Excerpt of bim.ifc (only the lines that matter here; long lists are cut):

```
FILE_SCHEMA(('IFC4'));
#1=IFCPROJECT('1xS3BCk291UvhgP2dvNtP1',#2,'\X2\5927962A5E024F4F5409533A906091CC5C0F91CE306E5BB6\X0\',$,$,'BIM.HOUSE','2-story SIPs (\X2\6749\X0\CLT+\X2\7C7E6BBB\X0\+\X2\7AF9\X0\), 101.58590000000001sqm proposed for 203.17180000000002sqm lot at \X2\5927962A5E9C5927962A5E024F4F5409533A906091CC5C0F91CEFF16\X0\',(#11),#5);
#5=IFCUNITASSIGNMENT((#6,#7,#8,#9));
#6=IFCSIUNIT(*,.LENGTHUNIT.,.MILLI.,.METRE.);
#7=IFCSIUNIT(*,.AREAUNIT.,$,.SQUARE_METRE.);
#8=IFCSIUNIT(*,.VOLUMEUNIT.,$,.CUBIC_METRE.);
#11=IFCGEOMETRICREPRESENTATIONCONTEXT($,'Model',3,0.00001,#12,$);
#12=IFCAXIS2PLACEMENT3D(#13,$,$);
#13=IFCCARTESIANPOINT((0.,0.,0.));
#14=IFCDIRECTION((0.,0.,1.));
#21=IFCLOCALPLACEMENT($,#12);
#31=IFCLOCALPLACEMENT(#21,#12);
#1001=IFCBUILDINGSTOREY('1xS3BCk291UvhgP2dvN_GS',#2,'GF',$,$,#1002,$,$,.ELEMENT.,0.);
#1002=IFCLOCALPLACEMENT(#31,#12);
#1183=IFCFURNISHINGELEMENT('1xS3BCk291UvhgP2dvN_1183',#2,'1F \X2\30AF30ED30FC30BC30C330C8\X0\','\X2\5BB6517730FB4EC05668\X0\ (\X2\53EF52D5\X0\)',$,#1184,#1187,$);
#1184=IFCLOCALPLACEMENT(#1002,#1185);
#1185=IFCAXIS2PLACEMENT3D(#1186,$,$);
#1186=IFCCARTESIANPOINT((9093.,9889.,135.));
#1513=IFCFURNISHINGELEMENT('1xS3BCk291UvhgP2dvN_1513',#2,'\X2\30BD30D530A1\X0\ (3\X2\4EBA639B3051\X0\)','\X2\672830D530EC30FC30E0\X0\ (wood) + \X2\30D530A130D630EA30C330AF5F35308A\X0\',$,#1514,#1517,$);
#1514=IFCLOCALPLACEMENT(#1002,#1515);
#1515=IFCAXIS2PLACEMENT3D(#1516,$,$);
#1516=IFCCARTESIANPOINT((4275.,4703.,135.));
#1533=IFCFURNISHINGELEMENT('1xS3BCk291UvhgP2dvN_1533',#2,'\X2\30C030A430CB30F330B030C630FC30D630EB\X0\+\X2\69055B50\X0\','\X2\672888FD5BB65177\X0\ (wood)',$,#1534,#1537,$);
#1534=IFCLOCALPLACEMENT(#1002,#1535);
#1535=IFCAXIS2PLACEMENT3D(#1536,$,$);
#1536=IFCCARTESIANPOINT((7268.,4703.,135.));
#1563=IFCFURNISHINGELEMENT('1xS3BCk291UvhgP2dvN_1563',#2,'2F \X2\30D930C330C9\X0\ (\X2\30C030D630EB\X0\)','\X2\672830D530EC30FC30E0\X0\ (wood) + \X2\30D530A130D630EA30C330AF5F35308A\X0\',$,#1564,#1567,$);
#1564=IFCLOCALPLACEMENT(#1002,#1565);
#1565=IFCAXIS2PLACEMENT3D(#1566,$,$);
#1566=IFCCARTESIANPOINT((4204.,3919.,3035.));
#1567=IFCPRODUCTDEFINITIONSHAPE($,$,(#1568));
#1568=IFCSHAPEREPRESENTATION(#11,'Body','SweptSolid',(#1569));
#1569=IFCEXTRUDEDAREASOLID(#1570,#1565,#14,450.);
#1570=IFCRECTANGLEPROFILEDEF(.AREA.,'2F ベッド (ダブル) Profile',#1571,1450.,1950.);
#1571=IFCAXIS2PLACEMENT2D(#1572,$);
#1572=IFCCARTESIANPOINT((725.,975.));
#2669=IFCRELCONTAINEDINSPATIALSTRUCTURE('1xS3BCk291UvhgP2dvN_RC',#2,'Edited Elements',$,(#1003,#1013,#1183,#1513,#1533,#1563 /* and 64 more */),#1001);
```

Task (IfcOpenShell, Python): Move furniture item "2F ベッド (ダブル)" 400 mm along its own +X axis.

```python
import ifcopenshell
import ifcopenshell.api.geometry
import ifcopenshell.util.placement
import ifcopenshell.util.unit

model = ifcopenshell.open("bim.ifc")
unit_scale = ifcopenshell.util.unit.calculate_unit_scale(model)

item = model.by_id(1563)
matrix = ifcopenshell.util.placement.get_local_placement(item.ObjectPlacement)
matrix[:3, 3] += matrix[:3, 0] * 0.4 / unit_scale
ifcopenshell.api.geometry.edit_object_placement(model, product=item, matrix=matrix, is_si=False)

print(ifcopenshell.util.placement.get_local_placement(item.ObjectPlacement).round(3) + 0.0)

model.write("bim-out.ifc")
```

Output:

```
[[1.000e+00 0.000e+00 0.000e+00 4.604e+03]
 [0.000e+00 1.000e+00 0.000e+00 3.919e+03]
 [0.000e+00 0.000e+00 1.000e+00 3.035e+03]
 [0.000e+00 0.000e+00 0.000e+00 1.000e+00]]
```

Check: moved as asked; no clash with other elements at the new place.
